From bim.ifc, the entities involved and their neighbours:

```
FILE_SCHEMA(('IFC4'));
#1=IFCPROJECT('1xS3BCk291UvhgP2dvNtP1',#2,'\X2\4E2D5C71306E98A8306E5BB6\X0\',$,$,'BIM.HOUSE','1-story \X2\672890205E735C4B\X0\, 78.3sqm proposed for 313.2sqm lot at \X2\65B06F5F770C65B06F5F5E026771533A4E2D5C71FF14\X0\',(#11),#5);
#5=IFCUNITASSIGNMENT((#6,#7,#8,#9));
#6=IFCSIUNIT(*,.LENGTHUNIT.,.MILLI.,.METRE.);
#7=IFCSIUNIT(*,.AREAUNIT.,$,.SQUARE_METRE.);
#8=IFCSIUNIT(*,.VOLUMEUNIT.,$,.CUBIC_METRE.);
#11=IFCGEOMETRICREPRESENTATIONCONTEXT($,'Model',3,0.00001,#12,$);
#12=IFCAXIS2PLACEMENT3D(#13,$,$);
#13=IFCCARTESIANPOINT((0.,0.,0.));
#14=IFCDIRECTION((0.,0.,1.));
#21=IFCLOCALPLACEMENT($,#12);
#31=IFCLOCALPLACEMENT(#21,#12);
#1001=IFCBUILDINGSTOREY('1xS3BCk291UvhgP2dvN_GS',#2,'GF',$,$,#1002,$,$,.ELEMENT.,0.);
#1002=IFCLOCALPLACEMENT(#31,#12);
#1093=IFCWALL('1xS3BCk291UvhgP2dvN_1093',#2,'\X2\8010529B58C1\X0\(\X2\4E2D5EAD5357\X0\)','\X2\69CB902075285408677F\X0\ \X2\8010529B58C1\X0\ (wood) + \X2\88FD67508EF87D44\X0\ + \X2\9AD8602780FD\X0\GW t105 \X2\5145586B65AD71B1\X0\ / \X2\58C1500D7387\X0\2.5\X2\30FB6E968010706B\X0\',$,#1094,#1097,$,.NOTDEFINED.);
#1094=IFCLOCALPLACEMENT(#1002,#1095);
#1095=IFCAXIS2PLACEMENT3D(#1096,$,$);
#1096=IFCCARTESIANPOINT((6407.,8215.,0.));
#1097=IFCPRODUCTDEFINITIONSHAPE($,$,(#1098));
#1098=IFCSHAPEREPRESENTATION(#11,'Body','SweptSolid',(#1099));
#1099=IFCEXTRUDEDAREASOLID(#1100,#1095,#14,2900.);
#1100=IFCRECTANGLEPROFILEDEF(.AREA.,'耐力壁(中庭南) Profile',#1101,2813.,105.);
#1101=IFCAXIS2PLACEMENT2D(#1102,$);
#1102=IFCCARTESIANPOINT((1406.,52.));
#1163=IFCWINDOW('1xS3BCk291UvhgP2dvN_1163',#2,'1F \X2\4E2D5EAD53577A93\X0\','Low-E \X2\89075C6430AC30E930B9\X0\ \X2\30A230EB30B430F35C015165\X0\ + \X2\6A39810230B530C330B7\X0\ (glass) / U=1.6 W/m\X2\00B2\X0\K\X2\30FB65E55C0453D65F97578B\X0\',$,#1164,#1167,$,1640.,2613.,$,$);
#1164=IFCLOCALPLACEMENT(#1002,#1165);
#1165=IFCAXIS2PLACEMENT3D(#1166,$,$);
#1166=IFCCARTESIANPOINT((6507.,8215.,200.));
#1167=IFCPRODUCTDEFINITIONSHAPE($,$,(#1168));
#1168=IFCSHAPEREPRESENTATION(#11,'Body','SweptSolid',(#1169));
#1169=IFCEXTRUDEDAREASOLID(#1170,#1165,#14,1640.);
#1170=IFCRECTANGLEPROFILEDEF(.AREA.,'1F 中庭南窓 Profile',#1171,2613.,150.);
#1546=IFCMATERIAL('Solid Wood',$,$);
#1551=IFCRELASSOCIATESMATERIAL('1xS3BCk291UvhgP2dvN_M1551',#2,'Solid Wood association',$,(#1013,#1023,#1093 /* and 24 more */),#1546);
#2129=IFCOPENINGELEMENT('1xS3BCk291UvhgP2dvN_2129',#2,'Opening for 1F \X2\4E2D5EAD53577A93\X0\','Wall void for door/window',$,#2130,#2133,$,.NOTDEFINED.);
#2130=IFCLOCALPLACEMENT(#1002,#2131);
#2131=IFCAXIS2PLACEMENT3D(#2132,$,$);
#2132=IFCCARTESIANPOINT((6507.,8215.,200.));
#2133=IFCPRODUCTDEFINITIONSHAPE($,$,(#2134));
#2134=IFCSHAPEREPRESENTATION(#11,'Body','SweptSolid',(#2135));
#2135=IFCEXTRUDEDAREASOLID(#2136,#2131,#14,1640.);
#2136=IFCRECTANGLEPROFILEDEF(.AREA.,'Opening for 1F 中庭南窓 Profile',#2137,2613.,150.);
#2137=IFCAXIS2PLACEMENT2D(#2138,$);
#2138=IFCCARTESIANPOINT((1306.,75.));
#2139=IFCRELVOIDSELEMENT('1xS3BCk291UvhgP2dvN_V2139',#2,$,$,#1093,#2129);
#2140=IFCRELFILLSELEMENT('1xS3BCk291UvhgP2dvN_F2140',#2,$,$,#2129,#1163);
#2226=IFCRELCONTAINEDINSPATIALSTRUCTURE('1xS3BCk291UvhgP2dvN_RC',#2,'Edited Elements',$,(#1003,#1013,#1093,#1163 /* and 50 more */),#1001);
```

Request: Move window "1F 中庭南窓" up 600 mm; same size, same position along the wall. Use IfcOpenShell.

```python
import numpy as np
import ifcopenshell
import ifcopenshell.api.geometry
import ifcopenshell.util.placement
import ifcopenshell.util.unit

model = ifcopenshell.open("bim.ifc")
unit_scale = ifcopenshell.util.unit.calculate_unit_scale(model)

window = model.by_guid("1xS3BCk291UvhgP2dvN_1163")
opening = window.FillsVoids[0].RelatingOpeningElement
dz = 0.6 / unit_scale

shift = np.array([0.0, 0.0, dz])
# The window is not placed relative to its opening, so move both.
for product in (opening, window):
    matrix = ifcopenshell.util.placement.get_local_placement(product.ObjectPlacement)
    matrix[:3, 3] += shift
    ifcopenshell.api.geometry.edit_object_placement(model, product=product, matrix=matrix, is_si=False)

print(f"moved by {dz * unit_scale:+.3f} m")

model.write("bim_v2.ifc")
```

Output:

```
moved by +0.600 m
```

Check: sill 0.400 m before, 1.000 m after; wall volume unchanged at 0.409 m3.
